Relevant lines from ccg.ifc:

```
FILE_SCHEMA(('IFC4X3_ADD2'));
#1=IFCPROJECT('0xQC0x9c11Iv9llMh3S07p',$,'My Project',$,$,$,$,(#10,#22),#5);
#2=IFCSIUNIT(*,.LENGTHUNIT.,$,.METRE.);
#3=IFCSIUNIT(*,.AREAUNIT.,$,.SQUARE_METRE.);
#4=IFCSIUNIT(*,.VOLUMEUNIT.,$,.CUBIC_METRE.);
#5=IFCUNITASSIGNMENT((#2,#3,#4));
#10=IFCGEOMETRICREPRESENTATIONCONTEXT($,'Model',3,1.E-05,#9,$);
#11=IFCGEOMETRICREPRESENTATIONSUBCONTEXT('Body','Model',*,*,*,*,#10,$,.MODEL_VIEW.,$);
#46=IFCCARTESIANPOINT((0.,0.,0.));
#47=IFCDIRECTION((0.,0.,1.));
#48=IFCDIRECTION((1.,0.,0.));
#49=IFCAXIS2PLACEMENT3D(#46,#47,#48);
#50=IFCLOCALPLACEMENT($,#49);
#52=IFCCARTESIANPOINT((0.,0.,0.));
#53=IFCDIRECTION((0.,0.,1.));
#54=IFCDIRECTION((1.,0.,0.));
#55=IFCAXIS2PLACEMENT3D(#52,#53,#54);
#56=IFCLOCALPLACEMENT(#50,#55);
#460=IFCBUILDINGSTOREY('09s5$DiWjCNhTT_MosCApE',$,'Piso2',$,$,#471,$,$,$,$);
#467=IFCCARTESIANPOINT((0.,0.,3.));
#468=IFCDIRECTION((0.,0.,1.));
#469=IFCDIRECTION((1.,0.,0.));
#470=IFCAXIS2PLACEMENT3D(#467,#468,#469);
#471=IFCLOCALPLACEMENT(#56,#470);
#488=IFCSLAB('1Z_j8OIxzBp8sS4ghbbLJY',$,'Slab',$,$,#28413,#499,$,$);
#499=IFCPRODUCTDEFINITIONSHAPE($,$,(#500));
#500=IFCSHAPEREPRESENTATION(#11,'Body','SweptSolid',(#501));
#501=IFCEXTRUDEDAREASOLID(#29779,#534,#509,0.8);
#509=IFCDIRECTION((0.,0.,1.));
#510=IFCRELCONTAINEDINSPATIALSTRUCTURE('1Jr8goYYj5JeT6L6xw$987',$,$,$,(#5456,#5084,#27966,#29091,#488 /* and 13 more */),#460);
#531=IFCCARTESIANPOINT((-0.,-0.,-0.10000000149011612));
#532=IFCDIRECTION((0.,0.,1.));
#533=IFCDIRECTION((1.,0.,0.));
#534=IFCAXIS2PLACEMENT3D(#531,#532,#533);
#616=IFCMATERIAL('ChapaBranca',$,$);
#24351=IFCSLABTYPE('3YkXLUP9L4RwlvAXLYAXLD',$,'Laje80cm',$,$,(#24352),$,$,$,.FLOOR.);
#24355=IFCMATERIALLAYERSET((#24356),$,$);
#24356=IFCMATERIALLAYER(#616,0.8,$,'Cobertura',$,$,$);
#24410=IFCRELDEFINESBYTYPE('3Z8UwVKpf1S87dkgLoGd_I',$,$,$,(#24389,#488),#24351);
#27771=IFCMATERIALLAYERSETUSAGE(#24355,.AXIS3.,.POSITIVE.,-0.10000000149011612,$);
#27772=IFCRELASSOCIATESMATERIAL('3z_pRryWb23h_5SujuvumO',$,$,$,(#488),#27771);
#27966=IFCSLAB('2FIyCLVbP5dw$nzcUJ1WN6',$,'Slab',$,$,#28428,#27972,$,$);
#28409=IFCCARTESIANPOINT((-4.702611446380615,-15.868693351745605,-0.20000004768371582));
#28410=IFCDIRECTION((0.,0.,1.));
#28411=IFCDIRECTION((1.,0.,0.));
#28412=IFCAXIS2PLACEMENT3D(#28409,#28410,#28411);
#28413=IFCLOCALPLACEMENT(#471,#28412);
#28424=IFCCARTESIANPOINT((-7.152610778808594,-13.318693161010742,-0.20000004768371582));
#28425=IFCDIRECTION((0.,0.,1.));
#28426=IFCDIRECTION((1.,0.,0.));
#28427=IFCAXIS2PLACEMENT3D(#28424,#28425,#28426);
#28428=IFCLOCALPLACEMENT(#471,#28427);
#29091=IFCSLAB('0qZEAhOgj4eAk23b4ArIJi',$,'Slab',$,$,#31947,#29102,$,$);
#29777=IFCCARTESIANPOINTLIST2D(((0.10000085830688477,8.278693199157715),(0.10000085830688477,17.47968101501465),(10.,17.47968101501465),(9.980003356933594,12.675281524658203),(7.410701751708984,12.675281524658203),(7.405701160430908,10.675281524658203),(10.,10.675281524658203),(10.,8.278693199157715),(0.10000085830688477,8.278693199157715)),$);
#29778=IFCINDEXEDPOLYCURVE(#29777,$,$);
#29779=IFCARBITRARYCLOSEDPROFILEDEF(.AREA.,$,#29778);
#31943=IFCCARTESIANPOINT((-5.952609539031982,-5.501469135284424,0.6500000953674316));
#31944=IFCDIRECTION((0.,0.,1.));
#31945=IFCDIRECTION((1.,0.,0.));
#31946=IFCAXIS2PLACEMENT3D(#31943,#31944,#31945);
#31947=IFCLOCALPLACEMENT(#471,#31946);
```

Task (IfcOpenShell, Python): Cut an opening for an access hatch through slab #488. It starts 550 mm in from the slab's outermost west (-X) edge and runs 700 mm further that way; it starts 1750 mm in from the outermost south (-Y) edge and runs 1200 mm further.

```python
import numpy as np
import ifcopenshell
import ifcopenshell.api.feature
import ifcopenshell.api.geometry
import ifcopenshell.api.root
import ifcopenshell.geom
import ifcopenshell.util.placement
import ifcopenshell.util.representation
import ifcopenshell.util.shape
import ifcopenshell.util.unit

model = ifcopenshell.open("ccg.ifc")
unit_scale = ifcopenshell.util.unit.calculate_unit_scale(model)
settings = ifcopenshell.geom.settings()


def volume(element):
    """Net volume in cubic metres, openings subtracted."""
    shape = ifcopenshell.geom.create_shape(settings, element)
    return ifcopenshell.util.shape.get_volume(shape.geometry)


slab = model.by_id(488)
before = volume(slab)

# Extent in the slab's own axes, in metres. The edges named are its -X and -Y sides.
slab_shape = ifcopenshell.geom.create_shape(settings, slab)
vertices = ifcopenshell.util.shape.get_vertices(slab_shape.geometry)
x_min, y_min, bottom = vertices.min(axis=0)
top = vertices[:, 2].max()

opening = ifcopenshell.api.root.create_entity(model, ifc_class="IfcOpeningElement", name="Access hatch opening", predefined_type="OPENING")
context = ifcopenshell.util.representation.get_context(model, "Model", "Body", "MODEL_VIEW")
width, depth = 0.7, 1.2
outline = [(0.0, 0.0), (width, 0.0), (width, depth), (0.0, depth), (0.0, 0.0)]
# Overshoot both faces by 50 mm so the cut is clean.
shape = ifcopenshell.api.geometry.add_slab_representation(
    model, context=context, depth=top - bottom + 0.1, polyline=outline
)
ifcopenshell.api.geometry.assign_representation(model, product=opening, representation=shape)

matrix = ifcopenshell.util.placement.get_local_placement(slab.ObjectPlacement)
matrix[:, 3] = matrix @ np.append(np.array([x_min + 0.55, y_min + 1.75, bottom - 0.05]) / unit_scale, 1.0)
ifcopenshell.api.geometry.edit_object_placement(model, product=opening, matrix=matrix, is_si=False)
ifcopenshell.api.feature.add_feature(model, feature=opening, element=slab)

after = volume(slab)

print(f"slab volume {before:.3f} -> {after:.3f} m3")

model.write("ccg_updated.ifc")
```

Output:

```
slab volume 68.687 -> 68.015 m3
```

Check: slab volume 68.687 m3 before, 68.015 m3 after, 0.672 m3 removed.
